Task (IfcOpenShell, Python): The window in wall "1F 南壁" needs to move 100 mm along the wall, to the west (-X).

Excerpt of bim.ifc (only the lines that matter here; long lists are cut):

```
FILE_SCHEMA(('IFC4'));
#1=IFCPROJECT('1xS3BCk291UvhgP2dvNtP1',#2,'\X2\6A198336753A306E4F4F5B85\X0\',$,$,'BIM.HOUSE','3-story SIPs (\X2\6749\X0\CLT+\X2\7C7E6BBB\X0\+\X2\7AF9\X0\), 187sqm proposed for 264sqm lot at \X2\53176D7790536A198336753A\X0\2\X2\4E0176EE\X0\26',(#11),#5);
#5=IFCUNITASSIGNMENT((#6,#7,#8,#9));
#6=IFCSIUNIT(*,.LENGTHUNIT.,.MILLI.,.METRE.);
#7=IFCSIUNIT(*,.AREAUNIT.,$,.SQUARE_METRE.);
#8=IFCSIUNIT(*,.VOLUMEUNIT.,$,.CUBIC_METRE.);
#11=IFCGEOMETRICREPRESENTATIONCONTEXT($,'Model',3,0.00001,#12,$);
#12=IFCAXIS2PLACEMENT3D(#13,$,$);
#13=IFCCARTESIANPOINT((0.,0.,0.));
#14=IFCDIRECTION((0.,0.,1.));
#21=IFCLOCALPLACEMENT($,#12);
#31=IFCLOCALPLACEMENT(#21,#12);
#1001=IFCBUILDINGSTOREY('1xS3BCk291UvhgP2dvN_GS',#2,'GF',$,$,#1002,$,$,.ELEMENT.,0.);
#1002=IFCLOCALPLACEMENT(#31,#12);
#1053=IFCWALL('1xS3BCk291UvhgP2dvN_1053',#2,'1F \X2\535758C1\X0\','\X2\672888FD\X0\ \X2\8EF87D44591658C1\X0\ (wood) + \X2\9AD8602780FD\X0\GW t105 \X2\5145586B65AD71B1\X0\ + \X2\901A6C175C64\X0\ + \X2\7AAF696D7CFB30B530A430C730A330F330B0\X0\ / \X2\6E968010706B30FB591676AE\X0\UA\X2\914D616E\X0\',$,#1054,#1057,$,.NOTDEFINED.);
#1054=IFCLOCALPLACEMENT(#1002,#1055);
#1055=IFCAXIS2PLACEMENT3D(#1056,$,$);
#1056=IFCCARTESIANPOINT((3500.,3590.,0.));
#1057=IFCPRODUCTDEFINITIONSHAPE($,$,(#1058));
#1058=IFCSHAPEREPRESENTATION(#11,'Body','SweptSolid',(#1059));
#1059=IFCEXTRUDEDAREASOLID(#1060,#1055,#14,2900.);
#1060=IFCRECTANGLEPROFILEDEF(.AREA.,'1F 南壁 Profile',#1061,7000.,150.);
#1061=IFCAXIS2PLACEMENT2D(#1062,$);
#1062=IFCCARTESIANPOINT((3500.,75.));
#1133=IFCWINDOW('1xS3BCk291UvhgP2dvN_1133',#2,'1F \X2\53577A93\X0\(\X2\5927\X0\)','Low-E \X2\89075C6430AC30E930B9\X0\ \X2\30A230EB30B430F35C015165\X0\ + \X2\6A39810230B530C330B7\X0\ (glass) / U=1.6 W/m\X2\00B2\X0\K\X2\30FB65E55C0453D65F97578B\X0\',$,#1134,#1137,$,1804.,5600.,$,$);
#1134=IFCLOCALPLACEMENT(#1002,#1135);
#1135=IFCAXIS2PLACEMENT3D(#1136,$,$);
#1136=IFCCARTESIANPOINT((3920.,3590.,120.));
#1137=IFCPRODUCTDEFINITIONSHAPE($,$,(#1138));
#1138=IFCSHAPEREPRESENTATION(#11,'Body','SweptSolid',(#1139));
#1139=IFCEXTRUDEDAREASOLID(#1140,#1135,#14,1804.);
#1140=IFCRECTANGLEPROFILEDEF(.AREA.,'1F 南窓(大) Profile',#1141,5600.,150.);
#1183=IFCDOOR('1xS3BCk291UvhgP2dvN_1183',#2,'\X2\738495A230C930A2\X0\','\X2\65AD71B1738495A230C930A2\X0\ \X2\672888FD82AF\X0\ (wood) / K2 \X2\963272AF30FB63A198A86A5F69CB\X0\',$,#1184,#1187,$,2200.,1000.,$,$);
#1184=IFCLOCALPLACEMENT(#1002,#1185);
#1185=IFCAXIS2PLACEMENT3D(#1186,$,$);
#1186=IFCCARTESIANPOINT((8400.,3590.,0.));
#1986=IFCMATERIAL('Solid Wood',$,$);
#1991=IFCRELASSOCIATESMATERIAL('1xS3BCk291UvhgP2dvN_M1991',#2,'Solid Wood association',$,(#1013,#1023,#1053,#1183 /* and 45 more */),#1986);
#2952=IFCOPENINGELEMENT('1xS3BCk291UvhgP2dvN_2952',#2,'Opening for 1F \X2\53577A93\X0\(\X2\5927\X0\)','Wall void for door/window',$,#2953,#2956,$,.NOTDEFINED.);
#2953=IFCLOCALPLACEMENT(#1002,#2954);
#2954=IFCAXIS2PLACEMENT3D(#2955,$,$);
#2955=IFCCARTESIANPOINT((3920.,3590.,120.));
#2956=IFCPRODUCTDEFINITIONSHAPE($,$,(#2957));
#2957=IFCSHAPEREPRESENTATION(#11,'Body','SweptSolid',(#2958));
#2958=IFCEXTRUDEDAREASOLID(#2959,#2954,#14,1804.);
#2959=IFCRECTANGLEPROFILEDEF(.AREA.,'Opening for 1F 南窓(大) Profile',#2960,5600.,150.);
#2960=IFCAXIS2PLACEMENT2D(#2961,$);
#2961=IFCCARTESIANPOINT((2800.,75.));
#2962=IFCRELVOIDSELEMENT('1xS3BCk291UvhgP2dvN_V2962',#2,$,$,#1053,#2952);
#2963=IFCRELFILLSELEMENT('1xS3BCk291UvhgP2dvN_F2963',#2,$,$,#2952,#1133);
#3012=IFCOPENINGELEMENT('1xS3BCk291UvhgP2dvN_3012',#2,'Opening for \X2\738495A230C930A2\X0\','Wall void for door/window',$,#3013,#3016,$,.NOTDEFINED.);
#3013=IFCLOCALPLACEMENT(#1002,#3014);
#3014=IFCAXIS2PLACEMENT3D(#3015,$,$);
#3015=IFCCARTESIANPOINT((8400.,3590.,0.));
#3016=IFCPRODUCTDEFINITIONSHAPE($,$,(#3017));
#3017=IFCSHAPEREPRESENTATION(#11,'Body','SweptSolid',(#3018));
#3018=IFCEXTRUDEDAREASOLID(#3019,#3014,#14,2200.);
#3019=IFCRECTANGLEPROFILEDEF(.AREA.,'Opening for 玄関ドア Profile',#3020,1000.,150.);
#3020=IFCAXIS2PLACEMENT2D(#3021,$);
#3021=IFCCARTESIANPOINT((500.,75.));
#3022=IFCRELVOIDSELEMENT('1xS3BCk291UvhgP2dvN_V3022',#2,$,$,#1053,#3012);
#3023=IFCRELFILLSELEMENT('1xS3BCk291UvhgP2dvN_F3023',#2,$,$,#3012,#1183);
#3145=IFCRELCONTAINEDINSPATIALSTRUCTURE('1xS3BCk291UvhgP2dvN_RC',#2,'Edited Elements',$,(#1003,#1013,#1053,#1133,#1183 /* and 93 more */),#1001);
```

```python
import ifcopenshell
import ifcopenshell.api.geometry
import ifcopenshell.util.placement

model = ifcopenshell.open("bim.ifc")

window = model.by_guid("1xS3BCk291UvhgP2dvN_1133")
opening = window.FillsVoids[0].RelatingOpeningElement
wall = opening.VoidsElements[0].RelatingBuildingElement

wall_matrix = ifcopenshell.util.placement.get_local_placement(wall.ObjectPlacement)
shift = wall_matrix[:3, 0] * -100.0
before = ifcopenshell.util.placement.get_local_placement(window.ObjectPlacement)[:3, 3].copy()

# The window is not placed relative to its opening, so move both.
for product in (opening, window):
    matrix = ifcopenshell.util.placement.get_local_placement(product.ObjectPlacement)
    matrix[:3, 3] += shift
    ifcopenshell.api.geometry.edit_object_placement(model, product=product, matrix=matrix, is_si=False)

after = ifcopenshell.util.placement.get_local_placement(window.ObjectPlacement)[:3, 3]
print("window moved by", (after - before).round(3) + 0.0)

model.write("bim-out.ifc")
```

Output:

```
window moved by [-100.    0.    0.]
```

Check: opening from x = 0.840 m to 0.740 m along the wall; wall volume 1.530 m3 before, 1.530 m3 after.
